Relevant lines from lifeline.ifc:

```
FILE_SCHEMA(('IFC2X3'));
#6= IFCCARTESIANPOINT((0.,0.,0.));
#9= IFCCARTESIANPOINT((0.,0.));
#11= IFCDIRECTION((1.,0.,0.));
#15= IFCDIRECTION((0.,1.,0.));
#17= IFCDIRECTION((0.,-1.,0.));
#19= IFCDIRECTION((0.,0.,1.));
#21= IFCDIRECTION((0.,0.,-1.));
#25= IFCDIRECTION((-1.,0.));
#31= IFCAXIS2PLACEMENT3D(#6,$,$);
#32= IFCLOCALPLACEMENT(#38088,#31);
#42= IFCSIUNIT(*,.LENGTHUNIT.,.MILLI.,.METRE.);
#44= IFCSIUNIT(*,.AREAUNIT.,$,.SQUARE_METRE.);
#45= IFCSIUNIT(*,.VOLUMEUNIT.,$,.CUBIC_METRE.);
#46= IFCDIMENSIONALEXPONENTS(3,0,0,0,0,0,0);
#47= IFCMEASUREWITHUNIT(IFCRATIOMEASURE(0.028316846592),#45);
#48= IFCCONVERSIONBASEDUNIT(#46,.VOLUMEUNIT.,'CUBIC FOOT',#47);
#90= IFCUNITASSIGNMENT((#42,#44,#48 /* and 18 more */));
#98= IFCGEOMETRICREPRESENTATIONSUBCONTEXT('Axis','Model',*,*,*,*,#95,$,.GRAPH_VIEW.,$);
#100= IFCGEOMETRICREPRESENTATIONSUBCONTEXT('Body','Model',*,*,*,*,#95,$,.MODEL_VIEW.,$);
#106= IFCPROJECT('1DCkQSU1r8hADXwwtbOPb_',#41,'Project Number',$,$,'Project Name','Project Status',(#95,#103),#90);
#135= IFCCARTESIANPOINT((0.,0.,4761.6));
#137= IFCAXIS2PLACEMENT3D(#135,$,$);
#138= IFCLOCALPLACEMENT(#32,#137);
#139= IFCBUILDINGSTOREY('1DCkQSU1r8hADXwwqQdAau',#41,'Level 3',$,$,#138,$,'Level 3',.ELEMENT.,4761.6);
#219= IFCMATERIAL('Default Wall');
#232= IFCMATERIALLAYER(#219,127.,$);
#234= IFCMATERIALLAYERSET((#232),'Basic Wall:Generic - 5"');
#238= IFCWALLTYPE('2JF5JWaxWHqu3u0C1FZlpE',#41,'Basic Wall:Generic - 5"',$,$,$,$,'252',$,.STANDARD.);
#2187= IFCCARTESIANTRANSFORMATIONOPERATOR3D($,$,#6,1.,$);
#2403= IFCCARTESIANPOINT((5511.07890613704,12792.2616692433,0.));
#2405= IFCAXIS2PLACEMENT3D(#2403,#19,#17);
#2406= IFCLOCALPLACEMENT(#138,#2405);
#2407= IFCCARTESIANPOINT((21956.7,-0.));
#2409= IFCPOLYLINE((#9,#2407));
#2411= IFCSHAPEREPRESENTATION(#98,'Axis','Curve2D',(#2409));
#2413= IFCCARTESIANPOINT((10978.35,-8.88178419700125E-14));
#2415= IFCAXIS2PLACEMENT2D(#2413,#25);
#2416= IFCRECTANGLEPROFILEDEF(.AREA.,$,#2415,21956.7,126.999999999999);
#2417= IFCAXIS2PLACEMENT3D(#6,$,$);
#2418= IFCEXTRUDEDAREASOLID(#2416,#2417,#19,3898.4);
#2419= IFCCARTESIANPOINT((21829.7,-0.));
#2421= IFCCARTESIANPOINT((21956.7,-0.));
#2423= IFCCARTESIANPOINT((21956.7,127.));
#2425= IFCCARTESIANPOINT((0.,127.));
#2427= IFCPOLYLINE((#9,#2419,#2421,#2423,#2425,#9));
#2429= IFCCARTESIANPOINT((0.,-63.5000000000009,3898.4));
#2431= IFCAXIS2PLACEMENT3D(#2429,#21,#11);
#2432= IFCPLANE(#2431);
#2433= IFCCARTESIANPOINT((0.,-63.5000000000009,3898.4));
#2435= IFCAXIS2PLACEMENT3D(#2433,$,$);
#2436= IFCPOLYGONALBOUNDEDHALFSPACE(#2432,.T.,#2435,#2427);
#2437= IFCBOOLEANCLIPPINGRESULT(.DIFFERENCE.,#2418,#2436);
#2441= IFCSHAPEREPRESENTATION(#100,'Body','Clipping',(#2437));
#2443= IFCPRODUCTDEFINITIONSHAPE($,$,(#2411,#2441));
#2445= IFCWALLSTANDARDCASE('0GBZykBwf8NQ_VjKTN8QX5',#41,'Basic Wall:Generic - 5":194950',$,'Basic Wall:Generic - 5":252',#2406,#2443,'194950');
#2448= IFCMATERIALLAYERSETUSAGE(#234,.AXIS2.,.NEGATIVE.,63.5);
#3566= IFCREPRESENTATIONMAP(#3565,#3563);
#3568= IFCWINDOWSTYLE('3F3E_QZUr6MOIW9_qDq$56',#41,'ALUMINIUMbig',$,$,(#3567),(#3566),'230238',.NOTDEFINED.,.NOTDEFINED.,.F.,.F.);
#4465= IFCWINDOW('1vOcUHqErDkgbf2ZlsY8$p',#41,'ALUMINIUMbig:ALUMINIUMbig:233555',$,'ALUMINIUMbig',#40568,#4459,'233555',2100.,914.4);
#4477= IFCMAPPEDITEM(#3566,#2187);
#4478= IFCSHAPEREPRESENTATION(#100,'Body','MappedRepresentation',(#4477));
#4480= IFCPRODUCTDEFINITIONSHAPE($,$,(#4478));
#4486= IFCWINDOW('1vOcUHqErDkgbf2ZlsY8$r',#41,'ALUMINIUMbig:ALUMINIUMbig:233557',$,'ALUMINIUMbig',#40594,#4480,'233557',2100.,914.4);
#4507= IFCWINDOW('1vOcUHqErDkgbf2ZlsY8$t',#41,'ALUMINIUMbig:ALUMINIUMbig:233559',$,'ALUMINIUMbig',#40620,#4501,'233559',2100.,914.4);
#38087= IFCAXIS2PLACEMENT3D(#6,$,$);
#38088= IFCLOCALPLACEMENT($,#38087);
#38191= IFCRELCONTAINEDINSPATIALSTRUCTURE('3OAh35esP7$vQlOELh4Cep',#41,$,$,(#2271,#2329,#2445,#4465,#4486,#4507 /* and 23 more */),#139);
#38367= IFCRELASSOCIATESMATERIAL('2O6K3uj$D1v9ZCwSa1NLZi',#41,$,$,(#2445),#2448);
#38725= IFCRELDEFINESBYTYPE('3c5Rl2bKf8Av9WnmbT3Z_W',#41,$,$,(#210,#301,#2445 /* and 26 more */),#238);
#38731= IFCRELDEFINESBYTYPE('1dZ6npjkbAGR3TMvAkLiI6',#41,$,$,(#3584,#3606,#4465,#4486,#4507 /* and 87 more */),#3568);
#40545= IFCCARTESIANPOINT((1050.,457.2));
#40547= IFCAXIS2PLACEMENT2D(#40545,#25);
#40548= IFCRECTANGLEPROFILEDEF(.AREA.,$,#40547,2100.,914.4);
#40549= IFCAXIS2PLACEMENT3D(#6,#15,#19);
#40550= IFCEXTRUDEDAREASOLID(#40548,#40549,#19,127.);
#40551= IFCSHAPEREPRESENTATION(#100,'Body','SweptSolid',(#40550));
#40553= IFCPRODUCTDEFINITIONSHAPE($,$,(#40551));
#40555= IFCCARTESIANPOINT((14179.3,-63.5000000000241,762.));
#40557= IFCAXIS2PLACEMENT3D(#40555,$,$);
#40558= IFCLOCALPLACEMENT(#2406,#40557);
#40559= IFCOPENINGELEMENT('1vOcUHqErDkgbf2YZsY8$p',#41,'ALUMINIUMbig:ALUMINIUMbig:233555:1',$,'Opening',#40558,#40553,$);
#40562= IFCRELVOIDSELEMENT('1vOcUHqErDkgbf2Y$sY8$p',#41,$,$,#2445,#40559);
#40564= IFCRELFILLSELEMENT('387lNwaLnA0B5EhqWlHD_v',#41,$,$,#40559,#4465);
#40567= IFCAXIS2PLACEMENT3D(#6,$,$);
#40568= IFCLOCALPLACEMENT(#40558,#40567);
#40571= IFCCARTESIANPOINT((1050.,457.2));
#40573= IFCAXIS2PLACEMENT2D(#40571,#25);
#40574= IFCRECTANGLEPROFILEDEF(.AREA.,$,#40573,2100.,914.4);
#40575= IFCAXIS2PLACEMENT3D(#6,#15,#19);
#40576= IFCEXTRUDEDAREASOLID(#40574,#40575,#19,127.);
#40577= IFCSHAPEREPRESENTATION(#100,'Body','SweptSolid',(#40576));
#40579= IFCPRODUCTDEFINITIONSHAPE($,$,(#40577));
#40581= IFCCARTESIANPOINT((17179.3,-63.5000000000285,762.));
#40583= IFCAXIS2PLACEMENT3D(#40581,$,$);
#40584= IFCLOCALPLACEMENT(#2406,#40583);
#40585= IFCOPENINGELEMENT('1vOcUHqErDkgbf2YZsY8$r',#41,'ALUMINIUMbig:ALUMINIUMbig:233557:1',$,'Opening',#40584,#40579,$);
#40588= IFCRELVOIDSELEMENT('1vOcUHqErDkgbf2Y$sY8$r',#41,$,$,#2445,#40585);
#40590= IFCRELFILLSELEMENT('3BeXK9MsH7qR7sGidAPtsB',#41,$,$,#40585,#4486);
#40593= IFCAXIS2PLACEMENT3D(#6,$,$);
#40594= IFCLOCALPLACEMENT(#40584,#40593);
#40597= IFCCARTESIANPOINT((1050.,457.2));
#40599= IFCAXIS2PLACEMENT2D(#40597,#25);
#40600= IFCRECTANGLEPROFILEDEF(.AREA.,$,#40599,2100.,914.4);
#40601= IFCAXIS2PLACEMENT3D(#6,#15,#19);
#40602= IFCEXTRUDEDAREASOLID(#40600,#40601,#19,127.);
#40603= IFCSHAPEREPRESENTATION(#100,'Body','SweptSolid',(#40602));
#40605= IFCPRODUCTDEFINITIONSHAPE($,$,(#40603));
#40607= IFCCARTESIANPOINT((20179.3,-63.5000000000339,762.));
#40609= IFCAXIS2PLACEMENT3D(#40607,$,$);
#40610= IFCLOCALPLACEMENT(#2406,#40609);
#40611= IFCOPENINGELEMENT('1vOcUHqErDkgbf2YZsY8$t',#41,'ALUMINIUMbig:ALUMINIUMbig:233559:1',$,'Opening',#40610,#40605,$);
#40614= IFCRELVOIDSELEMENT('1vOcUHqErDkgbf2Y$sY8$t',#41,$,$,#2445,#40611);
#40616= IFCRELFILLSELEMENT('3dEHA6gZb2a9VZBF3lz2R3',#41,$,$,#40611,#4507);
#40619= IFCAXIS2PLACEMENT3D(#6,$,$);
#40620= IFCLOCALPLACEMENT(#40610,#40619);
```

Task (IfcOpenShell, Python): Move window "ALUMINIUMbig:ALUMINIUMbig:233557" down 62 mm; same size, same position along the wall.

```python
import numpy as np
import ifcopenshell
import ifcopenshell.api.geometry
import ifcopenshell.util.placement
import ifcopenshell.util.unit

model = ifcopenshell.open("lifeline.ifc")
unit_scale = ifcopenshell.util.unit.calculate_unit_scale(model)

window = model.by_guid("1vOcUHqErDkgbf2ZlsY8$r")
opening = window.FillsVoids[0].RelatingOpeningElement
dz = -62.0

shift = np.array([0.0, 0.0, dz])
# The window is placed relative to its opening, so it follows when the opening moves.
matrix = ifcopenshell.util.placement.get_local_placement(opening.ObjectPlacement)
matrix[:3, 3] += shift
ifcopenshell.api.geometry.edit_object_placement(
    model, product=opening, matrix=matrix, is_si=False, should_transform_children=True
)

print(f"moved by {dz * unit_scale:+.3f} m")

model.write("lifeline_updated.ifc")
```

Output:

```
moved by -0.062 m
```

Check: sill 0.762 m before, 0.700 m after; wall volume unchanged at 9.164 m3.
